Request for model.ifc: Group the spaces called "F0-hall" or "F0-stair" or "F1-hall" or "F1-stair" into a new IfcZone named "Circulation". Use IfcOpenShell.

First a look at what the model holds.

```python
import ifcopenshell

model = ifcopenshell.open("model.ifc")
print(model.schema)
seen = {}
for space in model.by_type("IfcSpace"):
    seen[space.LongName] = seen.get(space.LongName, 0) + 1
for name, count in sorted(seen.items(), key=str):
    print(count, "x", name)
print("zones:", [z.Name for z in model.by_type("IfcZone")][:20])
```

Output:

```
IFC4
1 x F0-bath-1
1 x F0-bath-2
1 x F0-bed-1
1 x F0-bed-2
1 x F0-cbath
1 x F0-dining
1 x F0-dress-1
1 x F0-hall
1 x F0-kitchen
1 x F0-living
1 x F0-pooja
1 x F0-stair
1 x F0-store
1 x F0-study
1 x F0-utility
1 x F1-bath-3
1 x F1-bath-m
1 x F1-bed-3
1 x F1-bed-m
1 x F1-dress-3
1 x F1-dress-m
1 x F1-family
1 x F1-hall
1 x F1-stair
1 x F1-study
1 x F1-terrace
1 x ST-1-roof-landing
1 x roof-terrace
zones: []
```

```python
import ifcopenshell
import ifcopenshell.api.group
import ifcopenshell.api.root

model = ifcopenshell.open("model.ifc")

names = {"F0-hall", "F0-stair", "F1-hall", "F1-stair"}
spaces = [s for s in model.by_type("IfcSpace") if s.LongName in names]

zone = ifcopenshell.api.root.create_entity(model, ifc_class="IfcZone", name="Circulation")
ifcopenshell.api.group.assign_group(model, products=spaces, group=zone)
print(len(spaces), "spaces in", zone.Name)

model.write("model_rev.ifc")
```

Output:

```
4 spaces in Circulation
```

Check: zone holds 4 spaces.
